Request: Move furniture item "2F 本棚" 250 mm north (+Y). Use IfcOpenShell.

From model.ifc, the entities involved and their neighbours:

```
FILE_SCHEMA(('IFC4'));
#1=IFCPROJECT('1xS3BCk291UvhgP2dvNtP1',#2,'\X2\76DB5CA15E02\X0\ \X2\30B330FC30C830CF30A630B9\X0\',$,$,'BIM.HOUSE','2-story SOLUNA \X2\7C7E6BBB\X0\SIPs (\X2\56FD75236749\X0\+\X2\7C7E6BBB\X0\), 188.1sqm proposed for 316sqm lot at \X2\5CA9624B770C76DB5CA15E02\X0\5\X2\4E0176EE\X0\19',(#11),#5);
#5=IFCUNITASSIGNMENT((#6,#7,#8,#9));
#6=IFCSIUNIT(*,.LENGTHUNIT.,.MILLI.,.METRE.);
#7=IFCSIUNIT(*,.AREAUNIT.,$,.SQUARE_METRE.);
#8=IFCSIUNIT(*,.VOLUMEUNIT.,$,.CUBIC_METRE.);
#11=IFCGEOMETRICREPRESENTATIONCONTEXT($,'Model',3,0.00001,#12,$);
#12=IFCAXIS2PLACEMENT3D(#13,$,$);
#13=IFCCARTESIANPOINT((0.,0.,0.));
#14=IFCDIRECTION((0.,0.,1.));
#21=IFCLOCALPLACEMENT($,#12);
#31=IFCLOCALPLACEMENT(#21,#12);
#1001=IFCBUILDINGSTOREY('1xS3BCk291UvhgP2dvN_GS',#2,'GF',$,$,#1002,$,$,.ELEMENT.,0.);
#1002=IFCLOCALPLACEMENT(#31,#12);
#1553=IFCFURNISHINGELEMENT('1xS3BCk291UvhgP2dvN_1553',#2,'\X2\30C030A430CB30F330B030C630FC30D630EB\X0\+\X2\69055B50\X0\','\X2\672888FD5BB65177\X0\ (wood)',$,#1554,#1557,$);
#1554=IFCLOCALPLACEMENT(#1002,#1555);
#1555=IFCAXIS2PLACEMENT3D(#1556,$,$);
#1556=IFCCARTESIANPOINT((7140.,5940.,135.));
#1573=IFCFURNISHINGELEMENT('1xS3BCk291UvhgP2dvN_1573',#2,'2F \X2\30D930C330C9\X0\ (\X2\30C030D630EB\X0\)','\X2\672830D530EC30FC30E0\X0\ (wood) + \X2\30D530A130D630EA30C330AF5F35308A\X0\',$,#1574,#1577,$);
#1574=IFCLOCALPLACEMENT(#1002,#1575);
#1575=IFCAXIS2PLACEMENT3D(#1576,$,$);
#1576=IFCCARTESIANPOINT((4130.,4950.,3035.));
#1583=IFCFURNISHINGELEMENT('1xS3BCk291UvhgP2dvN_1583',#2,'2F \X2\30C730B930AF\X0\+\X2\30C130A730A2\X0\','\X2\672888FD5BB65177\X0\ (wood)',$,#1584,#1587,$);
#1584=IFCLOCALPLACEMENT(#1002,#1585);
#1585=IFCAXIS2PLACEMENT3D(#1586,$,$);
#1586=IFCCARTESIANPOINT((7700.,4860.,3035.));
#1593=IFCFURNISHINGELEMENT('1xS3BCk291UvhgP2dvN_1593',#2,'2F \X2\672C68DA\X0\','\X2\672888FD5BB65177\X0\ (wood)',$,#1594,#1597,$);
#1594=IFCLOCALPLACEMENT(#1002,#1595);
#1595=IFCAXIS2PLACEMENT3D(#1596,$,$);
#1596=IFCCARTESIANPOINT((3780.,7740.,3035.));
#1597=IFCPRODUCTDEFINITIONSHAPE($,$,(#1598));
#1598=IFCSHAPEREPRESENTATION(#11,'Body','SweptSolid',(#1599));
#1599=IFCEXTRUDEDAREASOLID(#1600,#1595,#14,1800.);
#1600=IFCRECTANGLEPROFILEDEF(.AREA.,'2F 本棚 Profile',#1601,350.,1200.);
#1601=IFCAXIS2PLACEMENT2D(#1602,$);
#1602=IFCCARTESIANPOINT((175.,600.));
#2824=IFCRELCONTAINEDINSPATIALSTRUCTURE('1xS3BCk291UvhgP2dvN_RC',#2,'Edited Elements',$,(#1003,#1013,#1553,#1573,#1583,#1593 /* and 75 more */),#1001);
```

```python
import ifcopenshell
import ifcopenshell.api.geometry
import ifcopenshell.util.placement

model = ifcopenshell.open("model.ifc")

item = model.by_guid("1xS3BCk291UvhgP2dvN_1593")
matrix = ifcopenshell.util.placement.get_local_placement(item.ObjectPlacement)
matrix[1, 3] += 250.0
ifcopenshell.api.geometry.edit_object_placement(model, product=item, matrix=matrix, is_si=False)

print(ifcopenshell.util.placement.get_local_placement(item.ObjectPlacement).round(3) + 0.0)

model.write("model_rev.ifc")
```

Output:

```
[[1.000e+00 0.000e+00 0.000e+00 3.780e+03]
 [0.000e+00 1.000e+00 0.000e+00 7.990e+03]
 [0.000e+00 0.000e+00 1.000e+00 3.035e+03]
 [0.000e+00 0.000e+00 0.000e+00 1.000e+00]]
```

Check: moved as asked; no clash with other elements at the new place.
